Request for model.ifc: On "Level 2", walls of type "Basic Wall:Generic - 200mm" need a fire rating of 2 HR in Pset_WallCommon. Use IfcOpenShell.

First a look at what the model holds.

```python
import ifcopenshell
import ifcopenshell.util.element

model = ifcopenshell.open("model.ifc")
print(model.schema)
storey = next(s for s in model.by_type("IfcBuildingStorey") if s.Name == "Level 2")
walls = [e for e in ifcopenshell.util.element.get_decomposition(storey) if e.is_a("IfcWall")]
seen = {}
for e in walls:
    element_type = ifcopenshell.util.element.get_type(e)
    key = (element_type.Name if element_type != e and element_type else None, ifcopenshell.util.element.get_pset(e, "Pset_WallCommon", "FireRating"))
    seen[key] = seen.get(key, 0) + 1
for (name, value), count in sorted(seen.items(), key=str):
    print(count, "x", name, "|", value)
```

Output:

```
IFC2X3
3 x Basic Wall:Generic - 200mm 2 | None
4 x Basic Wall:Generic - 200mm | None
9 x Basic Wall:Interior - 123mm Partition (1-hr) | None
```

```python
import ifcopenshell
import ifcopenshell.api.pset
import ifcopenshell.util.element

model = ifcopenshell.open("model.ifc")

storey = next(s for s in model.by_type("IfcBuildingStorey") if s.Name == "Level 2")
walls = [e for e in ifcopenshell.util.element.get_decomposition(storey) if e.is_a("IfcWall")]

count = 0
for e in walls:
    element_type = ifcopenshell.util.element.get_type(e)
    if element_type in (None, e) or element_type.Name != "Basic Wall:Generic - 200mm":
        continue
    found = ifcopenshell.util.element.get_pset(e, "Pset_WallCommon", should_inherit=False)
    if found:
        pset = model.by_id(found["id"])
        if len(ifcopenshell.util.element.get_elements_by_pset(pset)) > 1:
            pset = ifcopenshell.api.pset.unshare_pset(model, products=[e], pset=pset)[0]
    else:
        pset = ifcopenshell.api.pset.add_pset(model, product=e, name="Pset_WallCommon")
    ifcopenshell.api.pset.edit_pset(model, pset=pset, properties={"FireRating": "2 HR"})
    count += 1

print(count, "walls updated")

model.write("model_rev.ifc")
```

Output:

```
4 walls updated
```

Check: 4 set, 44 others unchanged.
